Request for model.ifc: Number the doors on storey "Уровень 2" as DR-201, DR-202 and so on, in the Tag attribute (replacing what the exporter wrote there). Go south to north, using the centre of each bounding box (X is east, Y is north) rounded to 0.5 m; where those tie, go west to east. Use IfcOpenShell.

First a look at what the model holds.

```python
import ifcopenshell
import ifcopenshell.util.element
import ifcopenshell.util.placement

model = ifcopenshell.open("model.ifc")
print(model.schema)
storey = next(s for s in model.by_type("IfcBuildingStorey") if s.Name == "Уровень 2")
doors = [e for e in ifcopenshell.util.element.get_decomposition(storey) if e.is_a("IfcDoor")]
for e in sorted(doors, key=lambda e: e.id()):
    origin = ifcopenshell.util.placement.get_local_placement(e.ObjectPlacement)[:3, 3]
    print(e.id(), e.Tag, e.Name, origin.round(2) + 0.0, sep=" | ")
```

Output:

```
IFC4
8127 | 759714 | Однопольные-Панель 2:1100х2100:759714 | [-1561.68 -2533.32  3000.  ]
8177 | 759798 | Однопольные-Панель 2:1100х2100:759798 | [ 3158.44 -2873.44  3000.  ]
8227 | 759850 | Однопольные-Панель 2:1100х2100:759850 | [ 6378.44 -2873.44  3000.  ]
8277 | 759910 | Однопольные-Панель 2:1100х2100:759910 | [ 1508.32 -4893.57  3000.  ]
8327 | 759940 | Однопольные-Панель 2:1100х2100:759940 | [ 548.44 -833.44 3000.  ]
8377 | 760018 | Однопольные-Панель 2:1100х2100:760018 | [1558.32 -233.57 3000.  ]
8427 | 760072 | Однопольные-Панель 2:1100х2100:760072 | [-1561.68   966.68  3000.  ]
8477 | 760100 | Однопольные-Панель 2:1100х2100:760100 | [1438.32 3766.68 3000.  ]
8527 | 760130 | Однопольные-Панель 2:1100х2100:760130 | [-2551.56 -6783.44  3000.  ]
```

```python
import ifcopenshell
import ifcopenshell.geom
import ifcopenshell.util.element
import ifcopenshell.util.shape

model = ifcopenshell.open("model.ifc")
settings = ifcopenshell.geom.settings()
settings.set("use-world-coords", True)


def centre(element):
    shape = ifcopenshell.geom.create_shape(settings, element)
    return ifcopenshell.util.shape.get_bbox_centroid(shape.geometry)


storey = next(s for s in model.by_type("IfcBuildingStorey") if s.Name == "Уровень 2")
doors = [e for e in ifcopenshell.util.element.get_decomposition(storey) if e.is_a("IfcDoor")]

# Insertion points can sit at a corner or the storey origin, so sort by the geometry (in metres).
centres = {e: centre(e) for e in doors}
doors.sort(key=lambda e: (round(centres[e][1] / 0.5), centres[e][0]))

for i, e in enumerate(doors, start=1):
    number = f"DR-2{i:02d}"
    e.Tag = number
    print(e.id(), number)

model.write("model_edited.ifc")
```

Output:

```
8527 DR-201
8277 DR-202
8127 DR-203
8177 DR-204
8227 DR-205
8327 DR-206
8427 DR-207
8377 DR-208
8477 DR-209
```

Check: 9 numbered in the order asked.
